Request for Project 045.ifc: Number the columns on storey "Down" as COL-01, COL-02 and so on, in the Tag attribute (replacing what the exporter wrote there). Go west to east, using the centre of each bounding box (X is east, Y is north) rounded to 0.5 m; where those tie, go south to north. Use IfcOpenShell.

First a look at what the model holds.

```python
import ifcopenshell
import ifcopenshell.util.element
import ifcopenshell.util.placement

model = ifcopenshell.open("Project 045.ifc")
print(model.schema)
storey = next(s for s in model.by_type("IfcBuildingStorey") if s.Name == "Down")
columns = [e for e in ifcopenshell.util.element.get_decomposition(storey) if e.is_a("IfcColumn")]
for e in sorted(columns, key=lambda e: e.id()):
    origin = ifcopenshell.util.placement.get_local_placement(e.ObjectPlacement)[:3, 3]
    print(e.id(), e.Tag, e.Name, origin.round(2) + 0.0, sep=" | ")
```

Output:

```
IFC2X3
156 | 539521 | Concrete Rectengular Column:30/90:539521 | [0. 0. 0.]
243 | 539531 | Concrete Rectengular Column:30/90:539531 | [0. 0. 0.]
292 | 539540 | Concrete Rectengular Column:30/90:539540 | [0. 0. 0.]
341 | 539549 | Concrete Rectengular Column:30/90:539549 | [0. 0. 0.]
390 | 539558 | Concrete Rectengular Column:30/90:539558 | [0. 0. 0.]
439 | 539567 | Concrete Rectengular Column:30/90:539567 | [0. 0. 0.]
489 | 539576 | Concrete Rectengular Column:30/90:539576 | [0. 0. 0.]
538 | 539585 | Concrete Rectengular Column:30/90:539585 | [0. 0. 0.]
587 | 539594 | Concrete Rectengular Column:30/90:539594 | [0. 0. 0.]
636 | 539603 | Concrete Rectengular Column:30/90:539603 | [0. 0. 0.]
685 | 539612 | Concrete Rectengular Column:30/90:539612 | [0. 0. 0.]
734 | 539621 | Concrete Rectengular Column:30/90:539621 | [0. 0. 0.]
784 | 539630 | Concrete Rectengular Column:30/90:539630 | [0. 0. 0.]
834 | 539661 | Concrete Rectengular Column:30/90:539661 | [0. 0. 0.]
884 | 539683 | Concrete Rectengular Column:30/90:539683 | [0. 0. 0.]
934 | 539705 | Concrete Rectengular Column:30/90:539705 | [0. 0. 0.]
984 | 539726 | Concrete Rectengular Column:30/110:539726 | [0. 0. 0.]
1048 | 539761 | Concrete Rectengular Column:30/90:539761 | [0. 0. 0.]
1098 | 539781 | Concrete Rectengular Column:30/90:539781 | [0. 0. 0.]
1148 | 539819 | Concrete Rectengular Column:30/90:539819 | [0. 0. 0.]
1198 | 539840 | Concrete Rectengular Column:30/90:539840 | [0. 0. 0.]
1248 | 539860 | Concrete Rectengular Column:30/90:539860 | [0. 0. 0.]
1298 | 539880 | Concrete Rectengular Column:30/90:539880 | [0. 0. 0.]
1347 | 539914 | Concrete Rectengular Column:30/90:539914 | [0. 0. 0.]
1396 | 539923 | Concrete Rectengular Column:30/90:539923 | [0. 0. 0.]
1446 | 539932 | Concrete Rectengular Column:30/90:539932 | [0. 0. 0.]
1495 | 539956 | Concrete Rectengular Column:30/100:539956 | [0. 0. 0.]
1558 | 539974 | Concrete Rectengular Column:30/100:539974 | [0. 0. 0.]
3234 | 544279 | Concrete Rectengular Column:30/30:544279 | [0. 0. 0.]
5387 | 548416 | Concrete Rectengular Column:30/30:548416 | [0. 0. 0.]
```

```python
import ifcopenshell
import ifcopenshell.geom
import ifcopenshell.util.element
import ifcopenshell.util.shape

model = ifcopenshell.open("Project 045.ifc")
settings = ifcopenshell.geom.settings()
settings.set("use-world-coords", True)


def centre(element):
    shape = ifcopenshell.geom.create_shape(settings, element)
    return ifcopenshell.util.shape.get_bbox_centroid(shape.geometry)


storey = next(s for s in model.by_type("IfcBuildingStorey") if s.Name == "Down")
columns = [e for e in ifcopenshell.util.element.get_decomposition(storey) if e.is_a("IfcColumn")]

# Insertion points can sit at a corner or the storey origin, so sort by the geometry (in metres).
centres = {e: centre(e) for e in columns}
columns.sort(key=lambda e: (round(centres[e][0] / 0.5), centres[e][1]))

for i, e in enumerate(columns, start=1):
    number = f"COL-{i:02d}"
    e.Tag = number
    print(e.id(), number)

model.write("Project 045_edited.ifc")
```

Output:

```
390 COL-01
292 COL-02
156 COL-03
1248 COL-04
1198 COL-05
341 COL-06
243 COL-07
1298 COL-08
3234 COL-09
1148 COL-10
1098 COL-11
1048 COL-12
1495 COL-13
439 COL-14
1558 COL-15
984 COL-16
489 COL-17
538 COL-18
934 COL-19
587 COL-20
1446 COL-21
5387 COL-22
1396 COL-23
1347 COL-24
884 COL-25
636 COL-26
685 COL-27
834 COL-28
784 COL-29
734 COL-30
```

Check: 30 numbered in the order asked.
